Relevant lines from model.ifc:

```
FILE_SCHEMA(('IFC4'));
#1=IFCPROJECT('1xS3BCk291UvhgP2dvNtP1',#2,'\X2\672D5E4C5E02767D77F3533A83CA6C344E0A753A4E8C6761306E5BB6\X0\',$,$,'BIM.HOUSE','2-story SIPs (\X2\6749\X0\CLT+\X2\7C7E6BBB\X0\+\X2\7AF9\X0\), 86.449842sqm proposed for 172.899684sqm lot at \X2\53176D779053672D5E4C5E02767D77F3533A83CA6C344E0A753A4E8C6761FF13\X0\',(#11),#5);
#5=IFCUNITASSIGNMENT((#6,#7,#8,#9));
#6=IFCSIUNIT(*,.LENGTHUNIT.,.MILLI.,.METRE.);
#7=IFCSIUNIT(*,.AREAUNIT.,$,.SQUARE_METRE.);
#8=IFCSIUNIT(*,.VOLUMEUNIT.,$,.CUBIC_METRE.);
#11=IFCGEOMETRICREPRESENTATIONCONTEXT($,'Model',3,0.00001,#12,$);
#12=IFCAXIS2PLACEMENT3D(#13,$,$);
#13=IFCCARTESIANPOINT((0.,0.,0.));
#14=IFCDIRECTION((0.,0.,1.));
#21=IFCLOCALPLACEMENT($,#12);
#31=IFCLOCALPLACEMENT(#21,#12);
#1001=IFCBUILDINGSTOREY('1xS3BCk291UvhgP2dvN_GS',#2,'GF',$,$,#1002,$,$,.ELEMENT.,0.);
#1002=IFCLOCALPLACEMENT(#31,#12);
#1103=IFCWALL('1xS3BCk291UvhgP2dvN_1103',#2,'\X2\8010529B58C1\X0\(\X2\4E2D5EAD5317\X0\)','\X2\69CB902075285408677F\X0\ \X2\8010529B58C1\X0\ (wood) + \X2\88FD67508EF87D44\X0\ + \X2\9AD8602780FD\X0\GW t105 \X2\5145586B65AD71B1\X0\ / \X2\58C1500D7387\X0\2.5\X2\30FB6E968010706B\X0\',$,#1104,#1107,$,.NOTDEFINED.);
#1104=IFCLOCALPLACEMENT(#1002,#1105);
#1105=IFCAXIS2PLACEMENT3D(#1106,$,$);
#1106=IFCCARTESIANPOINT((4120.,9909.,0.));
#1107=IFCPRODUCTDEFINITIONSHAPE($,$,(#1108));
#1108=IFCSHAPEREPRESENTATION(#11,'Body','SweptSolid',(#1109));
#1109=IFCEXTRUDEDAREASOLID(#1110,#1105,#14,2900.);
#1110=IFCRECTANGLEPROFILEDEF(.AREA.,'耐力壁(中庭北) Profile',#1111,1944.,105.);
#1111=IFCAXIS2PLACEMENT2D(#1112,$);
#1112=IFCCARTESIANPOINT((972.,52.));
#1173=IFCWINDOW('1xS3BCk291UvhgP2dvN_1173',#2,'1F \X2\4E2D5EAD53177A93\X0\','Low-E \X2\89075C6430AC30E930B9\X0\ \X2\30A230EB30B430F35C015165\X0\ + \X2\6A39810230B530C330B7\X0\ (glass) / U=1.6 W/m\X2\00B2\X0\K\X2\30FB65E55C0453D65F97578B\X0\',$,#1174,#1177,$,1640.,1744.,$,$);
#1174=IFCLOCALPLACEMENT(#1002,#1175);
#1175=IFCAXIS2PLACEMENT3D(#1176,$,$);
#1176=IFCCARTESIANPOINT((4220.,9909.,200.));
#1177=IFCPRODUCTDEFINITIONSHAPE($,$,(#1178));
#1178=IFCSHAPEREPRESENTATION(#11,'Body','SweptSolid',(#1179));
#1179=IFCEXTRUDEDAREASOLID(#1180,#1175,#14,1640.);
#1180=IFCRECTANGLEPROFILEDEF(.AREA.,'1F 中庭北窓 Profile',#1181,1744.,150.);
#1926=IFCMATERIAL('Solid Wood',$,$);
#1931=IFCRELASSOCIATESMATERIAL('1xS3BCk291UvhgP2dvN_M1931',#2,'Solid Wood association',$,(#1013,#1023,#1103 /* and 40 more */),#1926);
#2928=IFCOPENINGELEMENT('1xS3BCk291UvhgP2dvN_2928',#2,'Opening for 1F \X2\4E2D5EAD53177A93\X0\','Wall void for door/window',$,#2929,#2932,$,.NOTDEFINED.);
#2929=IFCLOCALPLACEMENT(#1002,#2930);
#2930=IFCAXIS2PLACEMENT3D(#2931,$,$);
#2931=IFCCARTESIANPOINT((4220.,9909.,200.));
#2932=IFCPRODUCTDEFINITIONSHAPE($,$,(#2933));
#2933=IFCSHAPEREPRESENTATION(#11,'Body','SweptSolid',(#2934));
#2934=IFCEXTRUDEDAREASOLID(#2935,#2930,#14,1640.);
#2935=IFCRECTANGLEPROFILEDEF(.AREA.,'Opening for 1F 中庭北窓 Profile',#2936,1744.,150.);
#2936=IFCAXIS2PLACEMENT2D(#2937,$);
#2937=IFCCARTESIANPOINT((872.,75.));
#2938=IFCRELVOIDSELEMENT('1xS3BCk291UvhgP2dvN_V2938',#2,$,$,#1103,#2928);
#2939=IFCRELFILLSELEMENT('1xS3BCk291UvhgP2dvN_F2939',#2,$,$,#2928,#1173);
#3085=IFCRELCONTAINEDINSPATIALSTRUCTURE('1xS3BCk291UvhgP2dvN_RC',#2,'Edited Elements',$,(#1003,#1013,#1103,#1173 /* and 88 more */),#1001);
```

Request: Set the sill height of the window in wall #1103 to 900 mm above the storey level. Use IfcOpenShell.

```python
import numpy as np
import ifcopenshell
import ifcopenshell.api.geometry
import ifcopenshell.geom
import ifcopenshell.util.element
import ifcopenshell.util.placement
import ifcopenshell.util.shape
import ifcopenshell.util.unit

model = ifcopenshell.open("model.ifc")
unit_scale = ifcopenshell.util.unit.calculate_unit_scale(model)

window = model.by_id(1173)
opening = window.FillsVoids[0].RelatingOpeningElement
storey = ifcopenshell.util.element.get_container(window, ifc_class="IfcBuildingStorey")
level = ifcopenshell.util.placement.get_local_placement(storey.ObjectPlacement)[2, 3]

# The opening's origin need not be at the sill, so measure its lowest point.
shape = ifcopenshell.geom.create_shape(ifcopenshell.geom.settings(), opening)
bottom = ifcopenshell.util.shape.get_shape_bottom_elevation(shape, shape.geometry) / unit_scale
dz = level + 0.9 / unit_scale - bottom

shift = np.array([0.0, 0.0, dz])
# The window is not placed relative to its opening, so move both.
for product in (opening, window):
    matrix = ifcopenshell.util.placement.get_local_placement(product.ObjectPlacement)
    matrix[:3, 3] += shift
    ifcopenshell.api.geometry.edit_object_placement(model, product=product, matrix=matrix, is_si=False)

print(f"moved by {dz * unit_scale:+.3f} m")

model.write("model_v2.ifc")
```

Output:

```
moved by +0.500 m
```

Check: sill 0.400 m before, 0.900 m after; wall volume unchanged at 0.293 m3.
